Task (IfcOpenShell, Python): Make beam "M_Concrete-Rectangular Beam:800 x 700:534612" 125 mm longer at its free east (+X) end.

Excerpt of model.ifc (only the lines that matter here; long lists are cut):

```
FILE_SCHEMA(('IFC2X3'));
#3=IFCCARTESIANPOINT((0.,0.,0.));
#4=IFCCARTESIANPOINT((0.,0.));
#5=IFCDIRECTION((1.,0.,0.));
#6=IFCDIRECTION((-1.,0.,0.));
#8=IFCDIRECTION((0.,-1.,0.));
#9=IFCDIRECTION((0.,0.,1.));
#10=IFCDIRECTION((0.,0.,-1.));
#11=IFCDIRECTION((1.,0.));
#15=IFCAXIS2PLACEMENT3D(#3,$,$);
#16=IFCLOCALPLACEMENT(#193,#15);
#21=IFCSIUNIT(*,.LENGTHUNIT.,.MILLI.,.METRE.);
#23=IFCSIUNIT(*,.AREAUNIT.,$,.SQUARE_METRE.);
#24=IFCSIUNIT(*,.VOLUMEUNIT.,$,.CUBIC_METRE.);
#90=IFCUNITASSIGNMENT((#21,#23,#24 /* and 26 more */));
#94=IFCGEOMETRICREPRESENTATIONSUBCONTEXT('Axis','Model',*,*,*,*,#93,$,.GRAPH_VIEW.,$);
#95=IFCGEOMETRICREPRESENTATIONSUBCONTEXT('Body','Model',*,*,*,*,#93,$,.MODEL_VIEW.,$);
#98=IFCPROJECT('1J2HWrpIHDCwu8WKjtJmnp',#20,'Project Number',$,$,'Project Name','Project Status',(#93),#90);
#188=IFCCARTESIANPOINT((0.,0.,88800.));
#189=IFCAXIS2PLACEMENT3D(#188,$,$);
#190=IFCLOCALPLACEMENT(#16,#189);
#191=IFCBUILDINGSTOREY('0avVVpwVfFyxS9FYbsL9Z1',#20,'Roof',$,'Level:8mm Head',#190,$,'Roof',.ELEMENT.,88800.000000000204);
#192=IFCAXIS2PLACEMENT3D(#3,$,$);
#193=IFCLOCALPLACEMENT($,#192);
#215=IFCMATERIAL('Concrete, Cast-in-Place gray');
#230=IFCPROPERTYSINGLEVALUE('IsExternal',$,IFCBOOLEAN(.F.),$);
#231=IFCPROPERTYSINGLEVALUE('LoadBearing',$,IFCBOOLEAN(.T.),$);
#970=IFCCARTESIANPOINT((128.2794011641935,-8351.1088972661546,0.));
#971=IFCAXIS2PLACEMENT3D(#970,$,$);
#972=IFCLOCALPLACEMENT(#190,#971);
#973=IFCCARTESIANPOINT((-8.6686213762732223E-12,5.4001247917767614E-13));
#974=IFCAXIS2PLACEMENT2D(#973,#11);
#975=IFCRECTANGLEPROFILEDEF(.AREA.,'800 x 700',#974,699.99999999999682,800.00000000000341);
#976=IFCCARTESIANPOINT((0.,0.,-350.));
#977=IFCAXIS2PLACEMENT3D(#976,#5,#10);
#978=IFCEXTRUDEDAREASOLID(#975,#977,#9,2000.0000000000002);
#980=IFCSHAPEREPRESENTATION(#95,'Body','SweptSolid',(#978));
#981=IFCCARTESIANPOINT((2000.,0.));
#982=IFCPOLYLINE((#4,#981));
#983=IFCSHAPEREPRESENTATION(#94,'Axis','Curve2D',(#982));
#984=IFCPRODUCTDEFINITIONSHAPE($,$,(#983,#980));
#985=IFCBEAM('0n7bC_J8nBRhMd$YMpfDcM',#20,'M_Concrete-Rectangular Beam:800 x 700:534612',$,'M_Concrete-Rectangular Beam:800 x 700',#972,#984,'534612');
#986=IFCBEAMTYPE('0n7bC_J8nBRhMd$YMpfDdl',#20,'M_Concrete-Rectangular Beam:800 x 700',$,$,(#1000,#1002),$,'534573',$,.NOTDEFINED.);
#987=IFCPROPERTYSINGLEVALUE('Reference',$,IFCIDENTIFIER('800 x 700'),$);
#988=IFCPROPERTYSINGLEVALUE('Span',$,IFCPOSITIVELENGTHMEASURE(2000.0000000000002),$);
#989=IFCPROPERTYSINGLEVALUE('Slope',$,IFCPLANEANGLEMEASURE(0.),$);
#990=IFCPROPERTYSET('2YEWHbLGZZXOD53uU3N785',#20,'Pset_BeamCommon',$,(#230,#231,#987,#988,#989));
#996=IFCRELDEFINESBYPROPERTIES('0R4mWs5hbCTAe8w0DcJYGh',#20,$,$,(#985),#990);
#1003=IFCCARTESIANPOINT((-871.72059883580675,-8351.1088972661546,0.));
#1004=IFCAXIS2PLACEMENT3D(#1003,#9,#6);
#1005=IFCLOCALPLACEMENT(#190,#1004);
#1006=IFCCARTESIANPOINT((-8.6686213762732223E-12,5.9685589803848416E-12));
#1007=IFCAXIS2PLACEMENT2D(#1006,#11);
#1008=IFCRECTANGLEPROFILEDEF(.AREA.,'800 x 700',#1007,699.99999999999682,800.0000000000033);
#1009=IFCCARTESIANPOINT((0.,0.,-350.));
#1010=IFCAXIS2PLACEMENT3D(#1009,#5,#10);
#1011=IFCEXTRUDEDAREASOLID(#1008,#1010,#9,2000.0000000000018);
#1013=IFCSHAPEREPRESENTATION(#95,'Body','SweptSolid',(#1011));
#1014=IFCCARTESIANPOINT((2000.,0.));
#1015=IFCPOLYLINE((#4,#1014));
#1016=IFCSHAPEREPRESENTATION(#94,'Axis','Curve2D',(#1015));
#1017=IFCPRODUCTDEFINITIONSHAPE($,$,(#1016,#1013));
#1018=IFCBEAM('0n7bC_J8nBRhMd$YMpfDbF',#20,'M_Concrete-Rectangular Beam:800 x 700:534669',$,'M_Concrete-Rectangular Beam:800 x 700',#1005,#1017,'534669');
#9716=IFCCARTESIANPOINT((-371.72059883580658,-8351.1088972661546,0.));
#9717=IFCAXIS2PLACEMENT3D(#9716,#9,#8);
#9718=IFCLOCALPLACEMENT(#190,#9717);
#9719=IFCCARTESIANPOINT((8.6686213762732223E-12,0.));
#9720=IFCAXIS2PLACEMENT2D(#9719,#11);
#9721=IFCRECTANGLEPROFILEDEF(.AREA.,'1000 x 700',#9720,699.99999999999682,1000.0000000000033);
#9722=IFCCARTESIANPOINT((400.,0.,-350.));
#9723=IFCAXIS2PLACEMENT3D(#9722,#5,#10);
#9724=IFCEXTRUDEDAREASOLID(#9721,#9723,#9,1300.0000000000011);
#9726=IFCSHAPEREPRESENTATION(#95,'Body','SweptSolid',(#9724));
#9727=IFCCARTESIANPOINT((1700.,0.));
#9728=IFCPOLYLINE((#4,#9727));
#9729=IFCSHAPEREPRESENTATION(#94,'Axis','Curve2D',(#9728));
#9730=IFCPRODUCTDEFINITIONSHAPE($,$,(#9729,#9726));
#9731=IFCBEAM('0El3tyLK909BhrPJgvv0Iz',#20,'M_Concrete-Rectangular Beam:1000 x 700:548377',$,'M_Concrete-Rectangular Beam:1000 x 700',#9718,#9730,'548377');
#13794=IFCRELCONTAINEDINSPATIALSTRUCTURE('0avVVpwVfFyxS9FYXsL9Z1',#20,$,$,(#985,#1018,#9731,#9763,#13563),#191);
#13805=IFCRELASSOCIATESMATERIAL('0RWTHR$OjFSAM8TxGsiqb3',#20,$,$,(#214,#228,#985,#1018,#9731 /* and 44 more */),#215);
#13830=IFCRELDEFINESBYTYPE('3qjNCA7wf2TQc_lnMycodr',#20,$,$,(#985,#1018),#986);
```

```python
import numpy as np
import ifcopenshell
import ifcopenshell.api.pset
import ifcopenshell.util.element
import ifcopenshell.util.representation

model = ifcopenshell.open("model.ifc")

member = model.by_guid("0n7bC_J8nBRhMd$YMpfDcM")
change = 125.0

# The extrusion runs towards the end named, so only its depth changes.
body = ifcopenshell.util.representation.get_representation(member, "Model", "Body")
solid = body.Items[0]
old_length = solid.Depth
solid.Depth += change

# Move the axis end point with it.
axis = next(r for r in member.Representation.Representations if r.RepresentationIdentifier == "Axis").Items[0]
start, end = (np.array(p.Coordinates) for p in axis.Points)
end = end + (end - start) / np.linalg.norm(end - start) * change
point = model.createIfcCartesianPoint(end.tolist())
axis.Points = [axis.Points[0], point]

# Update the stored length and volume.
pset = model.by_id(ifcopenshell.util.element.get_pset(member, "Pset_BeamCommon", should_inherit=False)["id"])
ifcopenshell.api.pset.edit_pset(model, pset=pset, properties={
    "Span": model.create_entity("IfcPositiveLengthMeasure", solid.Depth),
})

print(f"length {old_length:g} -> {solid.Depth:g}")

model.write("model_edited.ifc")
```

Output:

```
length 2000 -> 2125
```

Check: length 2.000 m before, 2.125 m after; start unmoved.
